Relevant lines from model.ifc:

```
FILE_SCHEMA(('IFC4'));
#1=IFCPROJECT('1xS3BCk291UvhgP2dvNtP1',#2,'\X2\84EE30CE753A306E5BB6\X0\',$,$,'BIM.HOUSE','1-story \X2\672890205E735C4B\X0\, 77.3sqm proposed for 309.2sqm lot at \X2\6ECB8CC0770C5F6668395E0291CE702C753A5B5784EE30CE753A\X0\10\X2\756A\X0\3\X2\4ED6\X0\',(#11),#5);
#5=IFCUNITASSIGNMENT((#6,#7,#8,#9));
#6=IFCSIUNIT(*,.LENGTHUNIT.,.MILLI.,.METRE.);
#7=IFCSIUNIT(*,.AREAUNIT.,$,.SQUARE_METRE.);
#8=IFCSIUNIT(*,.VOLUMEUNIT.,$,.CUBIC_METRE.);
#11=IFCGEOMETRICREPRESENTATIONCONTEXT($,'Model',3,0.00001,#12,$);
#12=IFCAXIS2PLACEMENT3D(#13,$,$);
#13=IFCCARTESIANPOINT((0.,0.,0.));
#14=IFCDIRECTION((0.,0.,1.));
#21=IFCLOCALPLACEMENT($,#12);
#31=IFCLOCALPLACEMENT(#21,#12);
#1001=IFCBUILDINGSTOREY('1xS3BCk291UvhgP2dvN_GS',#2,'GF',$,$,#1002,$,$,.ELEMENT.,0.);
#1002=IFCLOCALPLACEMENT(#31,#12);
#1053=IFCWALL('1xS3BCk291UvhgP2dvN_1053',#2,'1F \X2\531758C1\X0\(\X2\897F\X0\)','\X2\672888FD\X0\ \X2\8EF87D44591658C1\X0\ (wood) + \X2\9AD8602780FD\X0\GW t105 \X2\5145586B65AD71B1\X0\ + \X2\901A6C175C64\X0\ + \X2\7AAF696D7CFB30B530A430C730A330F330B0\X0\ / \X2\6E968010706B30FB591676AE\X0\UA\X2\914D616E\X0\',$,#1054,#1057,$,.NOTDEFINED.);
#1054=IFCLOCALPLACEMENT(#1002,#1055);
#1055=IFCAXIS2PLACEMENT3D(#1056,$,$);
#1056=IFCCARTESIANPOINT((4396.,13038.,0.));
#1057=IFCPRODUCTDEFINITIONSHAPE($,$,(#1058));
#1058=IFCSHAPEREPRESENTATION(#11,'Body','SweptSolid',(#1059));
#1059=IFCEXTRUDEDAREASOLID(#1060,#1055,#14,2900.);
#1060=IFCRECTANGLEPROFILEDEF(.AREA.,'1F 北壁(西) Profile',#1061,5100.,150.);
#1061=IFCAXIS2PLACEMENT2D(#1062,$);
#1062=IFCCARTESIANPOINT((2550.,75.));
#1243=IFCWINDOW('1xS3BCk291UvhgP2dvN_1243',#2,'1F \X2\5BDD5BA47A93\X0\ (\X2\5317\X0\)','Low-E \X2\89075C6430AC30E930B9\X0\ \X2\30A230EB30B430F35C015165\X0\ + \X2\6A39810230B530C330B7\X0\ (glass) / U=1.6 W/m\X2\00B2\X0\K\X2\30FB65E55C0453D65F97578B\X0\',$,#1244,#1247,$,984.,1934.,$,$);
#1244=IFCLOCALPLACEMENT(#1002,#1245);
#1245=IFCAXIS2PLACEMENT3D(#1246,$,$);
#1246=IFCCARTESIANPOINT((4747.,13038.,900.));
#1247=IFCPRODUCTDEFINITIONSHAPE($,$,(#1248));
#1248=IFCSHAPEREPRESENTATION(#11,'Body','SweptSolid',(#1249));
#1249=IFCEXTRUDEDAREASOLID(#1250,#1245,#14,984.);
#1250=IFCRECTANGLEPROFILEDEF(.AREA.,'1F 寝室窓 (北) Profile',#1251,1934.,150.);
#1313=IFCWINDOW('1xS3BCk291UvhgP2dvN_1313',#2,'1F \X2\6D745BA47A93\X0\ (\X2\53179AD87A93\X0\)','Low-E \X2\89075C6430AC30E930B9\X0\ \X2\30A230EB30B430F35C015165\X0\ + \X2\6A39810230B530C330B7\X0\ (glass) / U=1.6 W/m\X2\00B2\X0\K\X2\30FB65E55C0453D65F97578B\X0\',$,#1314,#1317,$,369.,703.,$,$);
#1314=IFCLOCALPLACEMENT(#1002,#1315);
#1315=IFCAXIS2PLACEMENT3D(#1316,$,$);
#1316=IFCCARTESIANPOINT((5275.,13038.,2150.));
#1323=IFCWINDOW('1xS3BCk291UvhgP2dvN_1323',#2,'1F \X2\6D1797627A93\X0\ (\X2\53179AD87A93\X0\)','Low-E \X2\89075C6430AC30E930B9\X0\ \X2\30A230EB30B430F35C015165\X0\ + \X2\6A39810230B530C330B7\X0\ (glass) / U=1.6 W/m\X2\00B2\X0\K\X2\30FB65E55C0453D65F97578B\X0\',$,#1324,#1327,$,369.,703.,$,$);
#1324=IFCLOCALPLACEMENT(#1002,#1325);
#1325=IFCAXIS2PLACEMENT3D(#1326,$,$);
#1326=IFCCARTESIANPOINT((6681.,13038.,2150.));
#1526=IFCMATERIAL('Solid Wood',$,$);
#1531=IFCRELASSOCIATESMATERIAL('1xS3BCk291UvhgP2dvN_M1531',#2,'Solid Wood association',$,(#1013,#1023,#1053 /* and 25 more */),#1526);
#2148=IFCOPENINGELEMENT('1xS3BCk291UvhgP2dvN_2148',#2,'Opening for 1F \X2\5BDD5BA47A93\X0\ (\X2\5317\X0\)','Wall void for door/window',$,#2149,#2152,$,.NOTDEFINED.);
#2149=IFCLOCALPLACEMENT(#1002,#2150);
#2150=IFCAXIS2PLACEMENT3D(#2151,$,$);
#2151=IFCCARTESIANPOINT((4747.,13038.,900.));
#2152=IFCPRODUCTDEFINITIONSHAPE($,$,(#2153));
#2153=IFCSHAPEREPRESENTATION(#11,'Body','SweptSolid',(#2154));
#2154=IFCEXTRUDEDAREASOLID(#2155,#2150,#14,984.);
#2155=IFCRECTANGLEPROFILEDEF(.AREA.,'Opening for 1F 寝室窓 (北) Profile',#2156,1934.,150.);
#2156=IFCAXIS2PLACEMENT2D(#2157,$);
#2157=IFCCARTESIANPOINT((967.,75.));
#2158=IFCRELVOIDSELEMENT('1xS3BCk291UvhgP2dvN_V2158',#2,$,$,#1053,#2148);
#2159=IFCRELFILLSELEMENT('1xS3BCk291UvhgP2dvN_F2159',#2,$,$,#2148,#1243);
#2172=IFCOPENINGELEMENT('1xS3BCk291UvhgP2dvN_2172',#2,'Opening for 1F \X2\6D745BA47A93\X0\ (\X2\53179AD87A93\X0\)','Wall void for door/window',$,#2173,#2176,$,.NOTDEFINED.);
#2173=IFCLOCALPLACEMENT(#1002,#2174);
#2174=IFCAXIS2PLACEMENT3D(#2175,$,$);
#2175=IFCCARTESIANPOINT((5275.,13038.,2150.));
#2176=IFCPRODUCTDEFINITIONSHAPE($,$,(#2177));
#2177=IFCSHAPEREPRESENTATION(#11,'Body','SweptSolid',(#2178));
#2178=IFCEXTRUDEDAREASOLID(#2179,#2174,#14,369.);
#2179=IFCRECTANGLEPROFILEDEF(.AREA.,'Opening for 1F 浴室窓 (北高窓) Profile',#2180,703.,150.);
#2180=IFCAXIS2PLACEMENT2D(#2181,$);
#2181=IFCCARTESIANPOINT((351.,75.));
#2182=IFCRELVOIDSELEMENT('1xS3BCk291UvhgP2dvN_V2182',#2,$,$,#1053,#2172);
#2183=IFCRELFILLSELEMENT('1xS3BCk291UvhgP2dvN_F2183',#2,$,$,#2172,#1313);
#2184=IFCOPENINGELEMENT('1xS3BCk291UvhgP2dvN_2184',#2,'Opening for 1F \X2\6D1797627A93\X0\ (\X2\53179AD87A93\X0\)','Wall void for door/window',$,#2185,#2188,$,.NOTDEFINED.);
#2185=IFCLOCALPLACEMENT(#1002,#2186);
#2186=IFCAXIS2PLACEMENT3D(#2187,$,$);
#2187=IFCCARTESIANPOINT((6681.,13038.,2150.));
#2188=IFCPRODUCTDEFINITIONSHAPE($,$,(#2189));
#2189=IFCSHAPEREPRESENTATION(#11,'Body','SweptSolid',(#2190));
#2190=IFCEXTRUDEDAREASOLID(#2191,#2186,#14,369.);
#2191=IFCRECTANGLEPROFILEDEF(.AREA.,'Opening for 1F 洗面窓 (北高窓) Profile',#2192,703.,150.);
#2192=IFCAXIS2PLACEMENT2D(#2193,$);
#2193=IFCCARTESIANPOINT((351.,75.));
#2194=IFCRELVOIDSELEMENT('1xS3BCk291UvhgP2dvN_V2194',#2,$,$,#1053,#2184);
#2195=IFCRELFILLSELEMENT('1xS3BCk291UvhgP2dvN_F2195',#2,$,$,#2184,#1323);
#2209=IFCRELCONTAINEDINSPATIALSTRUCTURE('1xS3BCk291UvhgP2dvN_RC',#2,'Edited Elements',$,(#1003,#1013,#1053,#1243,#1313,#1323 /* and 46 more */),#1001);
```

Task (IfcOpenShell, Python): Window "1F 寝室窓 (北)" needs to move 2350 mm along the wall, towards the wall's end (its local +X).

```python
import ifcopenshell
import ifcopenshell.api.geometry
import ifcopenshell.util.placement
import ifcopenshell.util.unit

model = ifcopenshell.open("model.ifc")
unit_scale = ifcopenshell.util.unit.calculate_unit_scale(model)

window = model.by_guid("1xS3BCk291UvhgP2dvN_1243")
opening = window.FillsVoids[0].RelatingOpeningElement
wall = opening.VoidsElements[0].RelatingBuildingElement

wall_matrix = ifcopenshell.util.placement.get_local_placement(wall.ObjectPlacement)
shift = wall_matrix[:3, 0] * 2.35 / unit_scale
before = ifcopenshell.util.placement.get_local_placement(window.ObjectPlacement)[:3, 3].copy()

# The window is not placed relative to its opening, so move both.
for product in (opening, window):
    matrix = ifcopenshell.util.placement.get_local_placement(product.ObjectPlacement)
    matrix[:3, 3] += shift
    ifcopenshell.api.geometry.edit_object_placement(model, product=product, matrix=matrix, is_si=False)

after = ifcopenshell.util.placement.get_local_placement(window.ObjectPlacement)[:3, 3]
print("window moved by", (after - before).round(3) + 0.0)

model.write("model-out.ifc")
```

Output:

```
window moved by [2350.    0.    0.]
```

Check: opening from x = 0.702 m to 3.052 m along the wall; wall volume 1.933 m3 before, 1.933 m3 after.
